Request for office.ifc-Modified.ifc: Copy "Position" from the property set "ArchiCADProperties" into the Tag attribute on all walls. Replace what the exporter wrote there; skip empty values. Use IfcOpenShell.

First a look at what the model holds.

```python
import ifcopenshell
import ifcopenshell.util.element

model = ifcopenshell.open("office.ifc-Modified.ifc")
print(model.schema)
walls = model.by_type("IfcWall")
print(len(walls), "walls")
for e in walls[:8]:
    source = ifcopenshell.util.element.get_pset(e, "ArchiCADProperties", "Position")
    target = e.Tag
    print(e.id(), repr(source), repr(target), sep=" | ")
```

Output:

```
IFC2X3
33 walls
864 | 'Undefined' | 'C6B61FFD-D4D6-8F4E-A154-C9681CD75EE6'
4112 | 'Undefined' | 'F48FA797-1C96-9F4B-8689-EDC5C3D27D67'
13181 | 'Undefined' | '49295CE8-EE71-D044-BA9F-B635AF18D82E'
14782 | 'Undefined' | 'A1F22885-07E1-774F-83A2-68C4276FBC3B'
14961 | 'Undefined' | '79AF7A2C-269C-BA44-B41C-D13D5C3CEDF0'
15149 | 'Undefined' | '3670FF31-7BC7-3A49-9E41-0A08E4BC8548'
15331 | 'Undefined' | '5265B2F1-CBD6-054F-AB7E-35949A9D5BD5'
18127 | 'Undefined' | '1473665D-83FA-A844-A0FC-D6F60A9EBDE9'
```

```python
import ifcopenshell
import ifcopenshell.util.element

model = ifcopenshell.open("office.ifc-Modified.ifc")

count = 0
for e in model.by_type("IfcWall"):
    value = ifcopenshell.util.element.get_pset(e, "ArchiCADProperties", "Position")
    current = e.Tag
    if not value or not value.strip() or current == value:
        continue
    e.Tag = value
    count += 1

print(count, "walls updated")

model.write("office.ifc-Modified_v2.ifc")
```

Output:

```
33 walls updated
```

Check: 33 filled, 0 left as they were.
